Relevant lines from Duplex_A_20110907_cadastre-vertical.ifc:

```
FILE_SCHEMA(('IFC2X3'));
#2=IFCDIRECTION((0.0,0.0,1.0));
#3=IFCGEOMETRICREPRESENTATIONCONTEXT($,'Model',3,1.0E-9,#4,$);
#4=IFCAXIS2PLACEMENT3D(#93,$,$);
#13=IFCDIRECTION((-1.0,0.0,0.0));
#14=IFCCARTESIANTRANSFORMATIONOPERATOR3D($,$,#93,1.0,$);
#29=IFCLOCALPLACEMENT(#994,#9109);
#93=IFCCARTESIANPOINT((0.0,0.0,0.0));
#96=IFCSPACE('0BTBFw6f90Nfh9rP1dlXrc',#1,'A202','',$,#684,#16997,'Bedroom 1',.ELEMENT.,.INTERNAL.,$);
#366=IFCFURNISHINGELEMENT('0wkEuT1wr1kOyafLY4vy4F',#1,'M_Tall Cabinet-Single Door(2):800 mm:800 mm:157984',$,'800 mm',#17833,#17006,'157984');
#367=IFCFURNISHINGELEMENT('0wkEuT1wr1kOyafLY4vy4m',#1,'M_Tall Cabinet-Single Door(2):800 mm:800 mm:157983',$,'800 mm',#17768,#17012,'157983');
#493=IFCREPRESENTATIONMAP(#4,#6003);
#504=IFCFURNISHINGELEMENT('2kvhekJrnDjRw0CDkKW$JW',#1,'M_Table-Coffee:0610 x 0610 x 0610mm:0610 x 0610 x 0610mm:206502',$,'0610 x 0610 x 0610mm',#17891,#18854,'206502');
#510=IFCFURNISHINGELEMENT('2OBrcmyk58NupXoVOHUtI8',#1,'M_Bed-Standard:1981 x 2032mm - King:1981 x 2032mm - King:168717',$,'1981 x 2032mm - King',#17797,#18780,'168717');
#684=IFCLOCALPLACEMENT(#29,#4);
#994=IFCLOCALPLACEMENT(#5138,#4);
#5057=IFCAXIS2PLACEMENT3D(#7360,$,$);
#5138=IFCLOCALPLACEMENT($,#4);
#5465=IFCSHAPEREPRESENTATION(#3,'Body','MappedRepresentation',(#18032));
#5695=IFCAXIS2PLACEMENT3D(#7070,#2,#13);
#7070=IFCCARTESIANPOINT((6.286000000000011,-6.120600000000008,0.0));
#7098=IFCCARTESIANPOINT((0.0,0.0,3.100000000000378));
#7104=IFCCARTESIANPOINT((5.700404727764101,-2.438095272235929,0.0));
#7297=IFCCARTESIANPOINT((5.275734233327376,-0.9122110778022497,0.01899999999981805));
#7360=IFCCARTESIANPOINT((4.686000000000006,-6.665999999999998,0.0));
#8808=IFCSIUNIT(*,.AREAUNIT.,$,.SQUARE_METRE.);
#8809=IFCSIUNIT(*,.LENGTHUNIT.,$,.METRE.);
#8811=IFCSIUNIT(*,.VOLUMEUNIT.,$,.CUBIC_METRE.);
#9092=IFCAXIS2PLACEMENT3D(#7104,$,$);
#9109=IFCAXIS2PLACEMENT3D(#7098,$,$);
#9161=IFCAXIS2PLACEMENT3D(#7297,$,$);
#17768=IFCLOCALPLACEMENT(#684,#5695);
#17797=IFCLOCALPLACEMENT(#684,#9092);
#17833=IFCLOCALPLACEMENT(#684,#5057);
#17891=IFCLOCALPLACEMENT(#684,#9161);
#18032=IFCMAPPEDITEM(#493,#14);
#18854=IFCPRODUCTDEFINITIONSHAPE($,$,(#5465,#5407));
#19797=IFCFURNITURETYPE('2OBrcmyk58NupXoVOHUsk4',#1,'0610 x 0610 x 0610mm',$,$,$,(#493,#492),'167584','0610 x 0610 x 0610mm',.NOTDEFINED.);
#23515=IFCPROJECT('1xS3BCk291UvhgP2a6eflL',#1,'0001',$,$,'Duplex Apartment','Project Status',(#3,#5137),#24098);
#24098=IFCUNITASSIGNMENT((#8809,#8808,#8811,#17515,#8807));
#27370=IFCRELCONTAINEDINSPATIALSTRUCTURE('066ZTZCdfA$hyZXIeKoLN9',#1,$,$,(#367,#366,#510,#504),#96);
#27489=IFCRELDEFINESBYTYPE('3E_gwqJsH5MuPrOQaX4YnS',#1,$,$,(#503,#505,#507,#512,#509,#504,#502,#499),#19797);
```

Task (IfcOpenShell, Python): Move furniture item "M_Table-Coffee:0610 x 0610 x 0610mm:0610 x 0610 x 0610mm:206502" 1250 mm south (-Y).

```python
import ifcopenshell
import ifcopenshell.api.geometry
import ifcopenshell.util.placement

model = ifcopenshell.open("Duplex_A_20110907_cadastre-vertical.ifc")

item = model.by_guid("2kvhekJrnDjRw0CDkKW$JW")
matrix = ifcopenshell.util.placement.get_local_placement(item.ObjectPlacement)
matrix[1, 3] -= 1.25
ifcopenshell.api.geometry.edit_object_placement(model, product=item, matrix=matrix, is_si=False)

print(ifcopenshell.util.placement.get_local_placement(item.ObjectPlacement).round(3) + 0.0)

model.write("Duplex_A_20110907_cadastre-vertical_v2.ifc")
```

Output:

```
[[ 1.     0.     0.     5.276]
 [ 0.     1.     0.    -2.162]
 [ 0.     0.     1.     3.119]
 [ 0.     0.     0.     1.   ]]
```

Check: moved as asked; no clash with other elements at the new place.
